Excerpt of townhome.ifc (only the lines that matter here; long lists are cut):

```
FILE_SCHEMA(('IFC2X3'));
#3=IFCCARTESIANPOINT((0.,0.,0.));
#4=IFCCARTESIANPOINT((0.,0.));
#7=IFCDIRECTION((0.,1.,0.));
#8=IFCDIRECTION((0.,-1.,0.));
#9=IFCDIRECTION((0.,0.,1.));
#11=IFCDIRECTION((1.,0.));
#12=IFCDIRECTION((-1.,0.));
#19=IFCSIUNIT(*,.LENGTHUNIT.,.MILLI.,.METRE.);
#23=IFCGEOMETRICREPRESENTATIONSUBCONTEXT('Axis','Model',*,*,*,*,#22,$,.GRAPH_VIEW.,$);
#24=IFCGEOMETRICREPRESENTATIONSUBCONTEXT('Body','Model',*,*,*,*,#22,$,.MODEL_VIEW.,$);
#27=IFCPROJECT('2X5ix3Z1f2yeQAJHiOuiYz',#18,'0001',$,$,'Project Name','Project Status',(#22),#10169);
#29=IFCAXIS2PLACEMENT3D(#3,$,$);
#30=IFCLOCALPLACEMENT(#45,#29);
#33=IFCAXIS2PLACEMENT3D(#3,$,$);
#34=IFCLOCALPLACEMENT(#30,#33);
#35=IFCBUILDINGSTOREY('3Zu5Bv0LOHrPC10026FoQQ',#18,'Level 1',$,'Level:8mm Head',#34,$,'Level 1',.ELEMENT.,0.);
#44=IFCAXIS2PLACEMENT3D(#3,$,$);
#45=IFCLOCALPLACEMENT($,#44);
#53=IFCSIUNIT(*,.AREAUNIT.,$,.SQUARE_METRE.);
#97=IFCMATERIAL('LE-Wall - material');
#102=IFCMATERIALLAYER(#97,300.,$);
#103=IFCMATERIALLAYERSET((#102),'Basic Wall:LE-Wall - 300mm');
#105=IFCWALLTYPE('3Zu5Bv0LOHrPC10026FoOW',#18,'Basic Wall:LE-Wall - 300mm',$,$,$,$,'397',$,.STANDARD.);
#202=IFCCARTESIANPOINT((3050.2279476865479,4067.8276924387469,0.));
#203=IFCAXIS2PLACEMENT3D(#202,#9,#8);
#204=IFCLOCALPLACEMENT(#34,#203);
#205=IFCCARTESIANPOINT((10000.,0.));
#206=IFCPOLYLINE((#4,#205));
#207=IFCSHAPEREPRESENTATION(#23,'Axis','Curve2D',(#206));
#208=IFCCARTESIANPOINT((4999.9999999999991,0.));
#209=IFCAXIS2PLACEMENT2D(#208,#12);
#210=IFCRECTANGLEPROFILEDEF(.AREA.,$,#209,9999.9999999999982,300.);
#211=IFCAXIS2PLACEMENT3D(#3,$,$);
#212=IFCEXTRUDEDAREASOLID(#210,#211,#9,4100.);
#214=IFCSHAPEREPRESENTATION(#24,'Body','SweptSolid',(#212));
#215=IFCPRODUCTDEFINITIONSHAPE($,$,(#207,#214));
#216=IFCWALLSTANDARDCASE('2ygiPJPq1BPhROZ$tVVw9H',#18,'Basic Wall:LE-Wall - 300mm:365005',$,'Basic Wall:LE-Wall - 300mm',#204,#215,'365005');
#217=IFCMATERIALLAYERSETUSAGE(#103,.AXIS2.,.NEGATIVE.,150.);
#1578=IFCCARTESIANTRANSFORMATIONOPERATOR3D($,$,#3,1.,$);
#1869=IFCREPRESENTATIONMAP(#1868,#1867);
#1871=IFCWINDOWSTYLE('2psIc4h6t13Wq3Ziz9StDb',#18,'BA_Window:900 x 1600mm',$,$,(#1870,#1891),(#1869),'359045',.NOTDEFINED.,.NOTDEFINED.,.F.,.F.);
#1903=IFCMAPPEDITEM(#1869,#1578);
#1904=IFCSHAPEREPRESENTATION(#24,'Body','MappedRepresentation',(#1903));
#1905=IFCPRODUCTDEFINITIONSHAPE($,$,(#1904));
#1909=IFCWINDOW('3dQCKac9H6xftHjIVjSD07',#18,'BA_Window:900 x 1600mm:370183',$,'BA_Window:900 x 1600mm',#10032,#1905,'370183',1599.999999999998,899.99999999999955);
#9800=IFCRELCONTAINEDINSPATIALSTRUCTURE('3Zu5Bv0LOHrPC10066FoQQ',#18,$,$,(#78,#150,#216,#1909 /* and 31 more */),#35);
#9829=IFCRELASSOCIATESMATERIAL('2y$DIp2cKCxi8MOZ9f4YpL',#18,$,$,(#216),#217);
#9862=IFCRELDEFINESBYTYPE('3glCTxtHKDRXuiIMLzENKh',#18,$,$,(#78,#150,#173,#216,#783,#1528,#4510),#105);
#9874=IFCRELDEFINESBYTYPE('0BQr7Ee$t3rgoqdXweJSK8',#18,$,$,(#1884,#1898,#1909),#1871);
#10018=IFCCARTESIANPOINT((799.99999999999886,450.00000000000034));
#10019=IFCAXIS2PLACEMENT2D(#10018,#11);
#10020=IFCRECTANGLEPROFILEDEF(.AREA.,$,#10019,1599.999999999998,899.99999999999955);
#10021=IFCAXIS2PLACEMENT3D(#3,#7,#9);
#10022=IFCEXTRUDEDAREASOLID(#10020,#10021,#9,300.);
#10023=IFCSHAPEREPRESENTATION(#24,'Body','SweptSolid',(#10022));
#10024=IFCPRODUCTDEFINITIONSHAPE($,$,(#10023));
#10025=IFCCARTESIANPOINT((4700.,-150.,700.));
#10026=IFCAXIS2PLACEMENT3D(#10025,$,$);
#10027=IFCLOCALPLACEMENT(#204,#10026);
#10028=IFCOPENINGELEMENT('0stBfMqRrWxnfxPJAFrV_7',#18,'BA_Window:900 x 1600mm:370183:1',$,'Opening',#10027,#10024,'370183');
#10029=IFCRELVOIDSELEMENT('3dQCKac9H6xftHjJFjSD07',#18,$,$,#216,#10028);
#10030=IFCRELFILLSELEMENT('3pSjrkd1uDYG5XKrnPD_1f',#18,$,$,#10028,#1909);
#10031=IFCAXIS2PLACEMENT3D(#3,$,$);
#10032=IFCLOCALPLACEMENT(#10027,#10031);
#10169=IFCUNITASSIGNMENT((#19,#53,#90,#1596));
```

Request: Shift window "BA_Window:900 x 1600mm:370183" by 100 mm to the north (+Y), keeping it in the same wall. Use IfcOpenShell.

```python
import ifcopenshell
import ifcopenshell.api.geometry
import ifcopenshell.util.placement
import ifcopenshell.util.unit

model = ifcopenshell.open("townhome.ifc")
unit_scale = ifcopenshell.util.unit.calculate_unit_scale(model)

window = model.by_guid("3dQCKac9H6xftHjIVjSD07")
opening = window.FillsVoids[0].RelatingOpeningElement
wall = opening.VoidsElements[0].RelatingBuildingElement

wall_matrix = ifcopenshell.util.placement.get_local_placement(wall.ObjectPlacement)
shift = wall_matrix[:3, 0] * -0.1 / unit_scale
before = ifcopenshell.util.placement.get_local_placement(window.ObjectPlacement)[:3, 3].copy()

# The window is placed relative to its opening, so it follows when the opening moves.
matrix = ifcopenshell.util.placement.get_local_placement(opening.ObjectPlacement)
matrix[:3, 3] += shift
ifcopenshell.api.geometry.edit_object_placement(
    model, product=opening, matrix=matrix, is_si=False, should_transform_children=True
)

after = ifcopenshell.util.placement.get_local_placement(window.ObjectPlacement)[:3, 3]
print("window moved by", (after - before).round(3) + 0.0)

model.write("townhome_edited.ifc")
```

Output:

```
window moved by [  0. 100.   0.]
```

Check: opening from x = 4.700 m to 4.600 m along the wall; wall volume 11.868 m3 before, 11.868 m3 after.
